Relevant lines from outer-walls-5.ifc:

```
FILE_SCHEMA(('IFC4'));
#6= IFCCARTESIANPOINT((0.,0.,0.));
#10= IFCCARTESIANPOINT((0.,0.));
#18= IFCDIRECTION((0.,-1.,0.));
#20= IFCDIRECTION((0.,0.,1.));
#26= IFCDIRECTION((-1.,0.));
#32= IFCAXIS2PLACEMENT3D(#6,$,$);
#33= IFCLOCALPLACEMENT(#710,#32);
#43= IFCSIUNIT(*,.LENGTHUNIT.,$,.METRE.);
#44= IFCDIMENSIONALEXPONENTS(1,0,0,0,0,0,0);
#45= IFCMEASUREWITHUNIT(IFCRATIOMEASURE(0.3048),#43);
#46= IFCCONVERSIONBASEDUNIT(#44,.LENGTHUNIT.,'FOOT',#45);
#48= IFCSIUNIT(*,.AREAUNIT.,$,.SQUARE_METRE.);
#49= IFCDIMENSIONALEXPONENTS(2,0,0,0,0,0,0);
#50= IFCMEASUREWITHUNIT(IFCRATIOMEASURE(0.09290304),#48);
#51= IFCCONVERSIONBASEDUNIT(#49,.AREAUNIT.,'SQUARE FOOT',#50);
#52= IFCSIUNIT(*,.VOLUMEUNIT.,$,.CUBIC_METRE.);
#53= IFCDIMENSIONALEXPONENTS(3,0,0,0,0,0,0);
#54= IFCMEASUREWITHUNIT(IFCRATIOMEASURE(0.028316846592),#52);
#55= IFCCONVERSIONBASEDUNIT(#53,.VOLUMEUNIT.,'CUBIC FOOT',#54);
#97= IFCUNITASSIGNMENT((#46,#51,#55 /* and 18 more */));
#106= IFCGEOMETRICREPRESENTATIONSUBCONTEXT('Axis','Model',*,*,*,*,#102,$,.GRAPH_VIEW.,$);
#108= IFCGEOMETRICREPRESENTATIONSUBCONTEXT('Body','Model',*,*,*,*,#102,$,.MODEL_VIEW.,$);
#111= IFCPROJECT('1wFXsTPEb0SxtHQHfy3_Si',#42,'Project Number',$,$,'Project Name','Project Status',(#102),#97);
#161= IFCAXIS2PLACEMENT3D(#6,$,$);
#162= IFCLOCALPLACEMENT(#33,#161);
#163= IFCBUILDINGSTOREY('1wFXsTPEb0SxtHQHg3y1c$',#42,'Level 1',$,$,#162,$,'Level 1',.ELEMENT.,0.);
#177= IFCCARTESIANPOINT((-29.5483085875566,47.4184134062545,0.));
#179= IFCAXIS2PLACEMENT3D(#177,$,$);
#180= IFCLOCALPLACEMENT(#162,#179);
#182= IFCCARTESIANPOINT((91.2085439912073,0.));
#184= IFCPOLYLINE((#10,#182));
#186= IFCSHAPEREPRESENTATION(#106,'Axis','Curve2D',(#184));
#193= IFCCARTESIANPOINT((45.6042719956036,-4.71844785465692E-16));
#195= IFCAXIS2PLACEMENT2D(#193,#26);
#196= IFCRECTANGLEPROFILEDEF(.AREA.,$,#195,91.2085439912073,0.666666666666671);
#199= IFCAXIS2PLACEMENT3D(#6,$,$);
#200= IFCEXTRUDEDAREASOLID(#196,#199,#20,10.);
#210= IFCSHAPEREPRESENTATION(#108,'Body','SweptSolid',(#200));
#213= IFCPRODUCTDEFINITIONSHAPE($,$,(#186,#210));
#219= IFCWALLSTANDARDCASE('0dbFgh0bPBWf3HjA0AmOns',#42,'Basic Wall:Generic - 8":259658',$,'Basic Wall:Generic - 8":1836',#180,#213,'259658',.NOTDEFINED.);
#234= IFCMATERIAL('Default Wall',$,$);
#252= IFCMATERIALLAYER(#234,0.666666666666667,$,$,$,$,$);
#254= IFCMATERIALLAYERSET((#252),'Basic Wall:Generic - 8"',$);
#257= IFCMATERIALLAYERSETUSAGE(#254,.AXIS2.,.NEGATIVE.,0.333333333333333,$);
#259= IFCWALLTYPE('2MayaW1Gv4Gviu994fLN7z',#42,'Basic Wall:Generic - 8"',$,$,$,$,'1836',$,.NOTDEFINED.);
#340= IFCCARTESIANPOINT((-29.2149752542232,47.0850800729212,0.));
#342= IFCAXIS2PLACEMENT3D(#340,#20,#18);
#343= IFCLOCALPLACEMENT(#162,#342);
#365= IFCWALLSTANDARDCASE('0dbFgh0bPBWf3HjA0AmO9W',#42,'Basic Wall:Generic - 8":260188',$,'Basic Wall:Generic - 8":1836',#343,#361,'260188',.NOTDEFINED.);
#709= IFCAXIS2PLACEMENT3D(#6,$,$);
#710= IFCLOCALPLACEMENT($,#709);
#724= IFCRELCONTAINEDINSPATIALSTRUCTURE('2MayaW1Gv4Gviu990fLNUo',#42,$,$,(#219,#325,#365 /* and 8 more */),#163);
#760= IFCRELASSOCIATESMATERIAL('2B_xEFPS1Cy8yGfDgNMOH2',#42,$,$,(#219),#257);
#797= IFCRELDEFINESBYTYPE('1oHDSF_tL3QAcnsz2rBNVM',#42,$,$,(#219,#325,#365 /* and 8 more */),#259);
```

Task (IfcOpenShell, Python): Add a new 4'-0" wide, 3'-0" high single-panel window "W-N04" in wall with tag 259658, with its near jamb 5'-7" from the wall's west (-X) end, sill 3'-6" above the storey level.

```python
import numpy as np
import ifcopenshell
import ifcopenshell.api.feature
import ifcopenshell.api.geometry
import ifcopenshell.api.root
import ifcopenshell.api.spatial
import ifcopenshell.geom
import ifcopenshell.util.element
import ifcopenshell.util.placement
import ifcopenshell.util.representation
import ifcopenshell.util.shape
import ifcopenshell.util.unit

model = ifcopenshell.open("outer-walls-5.ifc")
unit_scale = ifcopenshell.util.unit.calculate_unit_scale(model)
settings = ifcopenshell.geom.settings()


def volume(element):
    """Net volume in cubic metres, openings subtracted."""
    shape = ifcopenshell.geom.create_shape(settings, element)
    return ifcopenshell.util.shape.get_volume(shape.geometry)


wall = model.by_id(219)
storey = ifcopenshell.util.element.get_container(wall, ifc_class="IfcBuildingStorey")
context = ifcopenshell.util.representation.get_context(model, "Model", "Body", "MODEL_VIEW")
before = volume(wall)

width, height, from_end, sill = 1.2192, 0.9144, 1.7018, 1.0668  # metres

# The wall runs along its own X axis, and the end named is its -X end.
wall_shape = ifcopenshell.geom.create_shape(settings, wall)
x, y, z = ifcopenshell.util.shape.get_vertices(wall_shape.geometry).T
start = x.min() + from_end
face, thickness = float(y.min()), float(y.max() - y.min())
wall_matrix = ifcopenshell.util.placement.get_local_placement(wall.ObjectPlacement)
level = ifcopenshell.util.placement.get_local_placement(storey.ObjectPlacement)[2, 3]


def in_wall(x, y):
    """Placement at x, y metres in the wall's axes, at sill height."""
    matrix = wall_matrix.copy()
    matrix[:, 3] = wall_matrix @ np.array([x / unit_scale, y / unit_scale, 0.0, 1.0])
    matrix[2, 3] = level + sill / unit_scale
    return matrix


# Opening: a box that overshoots both wall faces by 50 mm.
opening = ifcopenshell.api.root.create_entity(model, ifc_class="IfcOpeningElement", predefined_type="OPENING")
box = ifcopenshell.api.geometry.add_wall_representation(
    model, context=context, length=width, height=height, thickness=thickness + 0.1
)
ifcopenshell.api.geometry.assign_representation(model, product=opening, representation=box)
ifcopenshell.api.geometry.edit_object_placement(model, product=opening, matrix=in_wall(start, face - 0.05), is_si=False)
ifcopenshell.api.feature.add_feature(model, feature=opening, element=wall)

window = ifcopenshell.api.root.create_entity(model, ifc_class="IfcWindow", name="W-N04", predefined_type="WINDOW")
window.OverallWidth, window.OverallHeight = width / unit_scale, height / unit_scale
window.PartitioningType = "SINGLE_PANEL"
body = ifcopenshell.api.geometry.add_window_representation(
    model,
    context=context,
    overall_width=window.OverallWidth,
    overall_height=window.OverallHeight,
    partition_type="SINGLE_PANEL",
)
ifcopenshell.api.geometry.assign_representation(model, product=window, representation=body)
ifcopenshell.api.spatial.assign_container(model, products=[window], relating_structure=storey)
ifcopenshell.api.feature.add_filling(model, opening=opening, element=window)

# Centre the window in the wall's thickness.
ifcopenshell.api.geometry.edit_object_placement(model, product=window, matrix=in_wall(start, face), is_si=False)
window_shape = ifcopenshell.geom.create_shape(settings, window)
depth = ifcopenshell.util.shape.get_vertices(window_shape.geometry)[:, 1]
offset = face + thickness / 2 - (depth.min() + depth.max()) / 2
ifcopenshell.api.geometry.edit_object_placement(model, product=window, matrix=in_wall(start, offset), is_si=False)

after = volume(wall)

print(f"wall volume {before:.3f} -> {after:.3f} m3")

model.write("outer-walls-5_rev.ifc")
```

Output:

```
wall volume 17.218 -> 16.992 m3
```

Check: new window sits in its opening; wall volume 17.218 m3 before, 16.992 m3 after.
